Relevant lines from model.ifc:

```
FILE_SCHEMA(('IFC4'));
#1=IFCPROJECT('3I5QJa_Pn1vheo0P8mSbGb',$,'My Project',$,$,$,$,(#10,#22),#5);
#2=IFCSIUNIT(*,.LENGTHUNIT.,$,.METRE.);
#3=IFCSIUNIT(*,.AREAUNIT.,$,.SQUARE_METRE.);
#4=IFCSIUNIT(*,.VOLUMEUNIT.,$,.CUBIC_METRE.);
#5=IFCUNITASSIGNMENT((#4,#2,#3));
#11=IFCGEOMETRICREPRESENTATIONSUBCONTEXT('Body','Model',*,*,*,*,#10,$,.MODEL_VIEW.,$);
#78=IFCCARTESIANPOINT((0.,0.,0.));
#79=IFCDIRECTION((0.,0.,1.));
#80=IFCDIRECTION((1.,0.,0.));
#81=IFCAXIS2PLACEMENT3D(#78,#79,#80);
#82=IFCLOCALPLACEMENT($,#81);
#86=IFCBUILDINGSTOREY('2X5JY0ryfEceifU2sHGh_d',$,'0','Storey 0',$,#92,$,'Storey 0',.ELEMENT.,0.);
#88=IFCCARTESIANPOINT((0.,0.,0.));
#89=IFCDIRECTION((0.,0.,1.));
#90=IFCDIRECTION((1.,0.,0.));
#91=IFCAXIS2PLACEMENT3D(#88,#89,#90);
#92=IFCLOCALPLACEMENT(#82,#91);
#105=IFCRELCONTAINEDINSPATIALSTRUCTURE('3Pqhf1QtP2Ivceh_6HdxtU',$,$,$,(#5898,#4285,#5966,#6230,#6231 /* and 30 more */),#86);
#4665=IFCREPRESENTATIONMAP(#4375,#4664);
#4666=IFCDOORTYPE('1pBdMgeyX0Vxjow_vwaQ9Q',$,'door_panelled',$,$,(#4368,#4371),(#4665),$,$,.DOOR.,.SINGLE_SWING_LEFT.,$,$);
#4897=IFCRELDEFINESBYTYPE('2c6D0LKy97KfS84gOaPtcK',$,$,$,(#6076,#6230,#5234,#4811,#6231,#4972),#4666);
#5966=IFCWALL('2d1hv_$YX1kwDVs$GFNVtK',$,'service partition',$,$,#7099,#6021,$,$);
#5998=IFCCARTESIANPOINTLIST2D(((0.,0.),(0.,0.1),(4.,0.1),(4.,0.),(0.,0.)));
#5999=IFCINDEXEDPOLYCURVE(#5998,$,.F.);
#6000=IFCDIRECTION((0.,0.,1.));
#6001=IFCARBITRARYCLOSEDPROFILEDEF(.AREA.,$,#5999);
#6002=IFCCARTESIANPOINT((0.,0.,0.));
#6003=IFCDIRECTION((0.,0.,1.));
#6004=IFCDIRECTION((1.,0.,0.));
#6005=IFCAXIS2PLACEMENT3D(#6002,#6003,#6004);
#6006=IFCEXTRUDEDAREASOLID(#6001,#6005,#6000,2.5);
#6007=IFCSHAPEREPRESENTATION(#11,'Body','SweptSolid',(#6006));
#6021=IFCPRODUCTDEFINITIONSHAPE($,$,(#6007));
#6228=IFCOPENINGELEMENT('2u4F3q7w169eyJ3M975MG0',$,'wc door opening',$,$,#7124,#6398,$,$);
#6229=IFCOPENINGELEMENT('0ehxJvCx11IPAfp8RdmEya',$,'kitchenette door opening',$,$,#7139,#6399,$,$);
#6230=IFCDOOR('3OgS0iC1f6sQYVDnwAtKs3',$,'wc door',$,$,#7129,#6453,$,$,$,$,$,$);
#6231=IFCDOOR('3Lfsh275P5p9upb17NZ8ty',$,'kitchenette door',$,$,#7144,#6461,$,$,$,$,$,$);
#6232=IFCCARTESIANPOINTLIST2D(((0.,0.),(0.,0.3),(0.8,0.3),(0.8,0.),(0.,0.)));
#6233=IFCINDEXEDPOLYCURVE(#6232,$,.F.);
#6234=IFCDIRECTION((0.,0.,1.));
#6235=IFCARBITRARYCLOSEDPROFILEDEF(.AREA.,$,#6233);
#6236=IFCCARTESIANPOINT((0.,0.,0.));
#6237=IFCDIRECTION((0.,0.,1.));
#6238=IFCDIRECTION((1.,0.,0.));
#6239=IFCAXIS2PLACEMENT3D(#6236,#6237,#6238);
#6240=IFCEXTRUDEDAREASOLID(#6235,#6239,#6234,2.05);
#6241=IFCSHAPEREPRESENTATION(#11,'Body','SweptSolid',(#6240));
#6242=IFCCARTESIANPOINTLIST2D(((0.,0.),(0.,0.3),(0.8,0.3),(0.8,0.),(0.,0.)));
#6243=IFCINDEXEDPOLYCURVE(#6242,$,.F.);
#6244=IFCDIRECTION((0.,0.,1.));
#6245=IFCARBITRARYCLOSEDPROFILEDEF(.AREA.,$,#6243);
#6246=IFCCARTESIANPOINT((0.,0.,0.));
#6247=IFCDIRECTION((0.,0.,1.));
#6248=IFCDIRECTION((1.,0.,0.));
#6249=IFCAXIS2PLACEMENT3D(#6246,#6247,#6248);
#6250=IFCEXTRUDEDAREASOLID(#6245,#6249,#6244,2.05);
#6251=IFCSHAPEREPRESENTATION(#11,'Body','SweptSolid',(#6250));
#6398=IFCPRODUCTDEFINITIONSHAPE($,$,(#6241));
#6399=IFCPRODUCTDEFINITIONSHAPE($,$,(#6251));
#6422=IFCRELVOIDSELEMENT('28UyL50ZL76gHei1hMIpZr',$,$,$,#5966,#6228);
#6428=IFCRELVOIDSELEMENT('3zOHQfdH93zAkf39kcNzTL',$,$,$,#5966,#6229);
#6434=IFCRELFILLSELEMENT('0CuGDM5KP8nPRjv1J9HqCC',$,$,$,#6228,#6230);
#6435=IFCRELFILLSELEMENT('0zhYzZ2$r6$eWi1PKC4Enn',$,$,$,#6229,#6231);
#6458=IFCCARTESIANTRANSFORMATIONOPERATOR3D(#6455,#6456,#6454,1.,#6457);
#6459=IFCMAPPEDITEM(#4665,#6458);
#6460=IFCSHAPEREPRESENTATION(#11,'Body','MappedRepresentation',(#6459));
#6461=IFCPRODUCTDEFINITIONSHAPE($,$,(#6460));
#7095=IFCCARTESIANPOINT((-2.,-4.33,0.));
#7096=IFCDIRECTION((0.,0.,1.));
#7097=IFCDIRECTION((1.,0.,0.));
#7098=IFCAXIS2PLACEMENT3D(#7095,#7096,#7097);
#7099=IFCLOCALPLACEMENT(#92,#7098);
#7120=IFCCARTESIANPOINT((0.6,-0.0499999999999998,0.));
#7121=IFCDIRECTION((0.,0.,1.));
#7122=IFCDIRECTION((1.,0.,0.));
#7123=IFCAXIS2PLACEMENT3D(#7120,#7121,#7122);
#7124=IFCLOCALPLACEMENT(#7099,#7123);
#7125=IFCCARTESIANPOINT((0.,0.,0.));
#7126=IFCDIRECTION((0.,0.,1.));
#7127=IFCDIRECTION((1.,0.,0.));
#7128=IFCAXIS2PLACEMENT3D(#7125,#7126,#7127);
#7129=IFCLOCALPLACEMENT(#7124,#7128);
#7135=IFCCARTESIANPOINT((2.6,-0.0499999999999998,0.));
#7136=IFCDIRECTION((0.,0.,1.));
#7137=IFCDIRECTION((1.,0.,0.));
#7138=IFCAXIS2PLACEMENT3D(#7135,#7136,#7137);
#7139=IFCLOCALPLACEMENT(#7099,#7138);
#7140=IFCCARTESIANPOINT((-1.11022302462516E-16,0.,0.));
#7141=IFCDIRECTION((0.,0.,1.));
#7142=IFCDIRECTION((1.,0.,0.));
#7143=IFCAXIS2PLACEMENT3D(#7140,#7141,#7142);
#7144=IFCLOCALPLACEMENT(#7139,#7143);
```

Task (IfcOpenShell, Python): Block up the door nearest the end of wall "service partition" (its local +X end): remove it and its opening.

```python
import ifcopenshell
import ifcopenshell.api.feature
import ifcopenshell.api.root
import ifcopenshell.geom
import ifcopenshell.util.shape

model = ifcopenshell.open("model.ifc")
settings = ifcopenshell.geom.settings()


def volume(element):
    """Net volume in cubic metres, openings subtracted."""
    shape = ifcopenshell.geom.create_shape(settings, element)
    return ifcopenshell.util.shape.get_volume(shape.geometry)


door = model.by_guid("3Lfsh275P5p9upb17NZ8ty")
opening = door.FillsVoids[0].RelatingOpeningElement
wall = opening.VoidsElements[0].RelatingBuildingElement
before = volume(wall)

ifcopenshell.api.root.remove_product(model, product=door)
ifcopenshell.api.feature.remove_feature(model, feature=opening)

after = volume(wall)

print(f"wall volume {before:.3f} -> {after:.3f} m3")

model.write("model_updated.ifc")
```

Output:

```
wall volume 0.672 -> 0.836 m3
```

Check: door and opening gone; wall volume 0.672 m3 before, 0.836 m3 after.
